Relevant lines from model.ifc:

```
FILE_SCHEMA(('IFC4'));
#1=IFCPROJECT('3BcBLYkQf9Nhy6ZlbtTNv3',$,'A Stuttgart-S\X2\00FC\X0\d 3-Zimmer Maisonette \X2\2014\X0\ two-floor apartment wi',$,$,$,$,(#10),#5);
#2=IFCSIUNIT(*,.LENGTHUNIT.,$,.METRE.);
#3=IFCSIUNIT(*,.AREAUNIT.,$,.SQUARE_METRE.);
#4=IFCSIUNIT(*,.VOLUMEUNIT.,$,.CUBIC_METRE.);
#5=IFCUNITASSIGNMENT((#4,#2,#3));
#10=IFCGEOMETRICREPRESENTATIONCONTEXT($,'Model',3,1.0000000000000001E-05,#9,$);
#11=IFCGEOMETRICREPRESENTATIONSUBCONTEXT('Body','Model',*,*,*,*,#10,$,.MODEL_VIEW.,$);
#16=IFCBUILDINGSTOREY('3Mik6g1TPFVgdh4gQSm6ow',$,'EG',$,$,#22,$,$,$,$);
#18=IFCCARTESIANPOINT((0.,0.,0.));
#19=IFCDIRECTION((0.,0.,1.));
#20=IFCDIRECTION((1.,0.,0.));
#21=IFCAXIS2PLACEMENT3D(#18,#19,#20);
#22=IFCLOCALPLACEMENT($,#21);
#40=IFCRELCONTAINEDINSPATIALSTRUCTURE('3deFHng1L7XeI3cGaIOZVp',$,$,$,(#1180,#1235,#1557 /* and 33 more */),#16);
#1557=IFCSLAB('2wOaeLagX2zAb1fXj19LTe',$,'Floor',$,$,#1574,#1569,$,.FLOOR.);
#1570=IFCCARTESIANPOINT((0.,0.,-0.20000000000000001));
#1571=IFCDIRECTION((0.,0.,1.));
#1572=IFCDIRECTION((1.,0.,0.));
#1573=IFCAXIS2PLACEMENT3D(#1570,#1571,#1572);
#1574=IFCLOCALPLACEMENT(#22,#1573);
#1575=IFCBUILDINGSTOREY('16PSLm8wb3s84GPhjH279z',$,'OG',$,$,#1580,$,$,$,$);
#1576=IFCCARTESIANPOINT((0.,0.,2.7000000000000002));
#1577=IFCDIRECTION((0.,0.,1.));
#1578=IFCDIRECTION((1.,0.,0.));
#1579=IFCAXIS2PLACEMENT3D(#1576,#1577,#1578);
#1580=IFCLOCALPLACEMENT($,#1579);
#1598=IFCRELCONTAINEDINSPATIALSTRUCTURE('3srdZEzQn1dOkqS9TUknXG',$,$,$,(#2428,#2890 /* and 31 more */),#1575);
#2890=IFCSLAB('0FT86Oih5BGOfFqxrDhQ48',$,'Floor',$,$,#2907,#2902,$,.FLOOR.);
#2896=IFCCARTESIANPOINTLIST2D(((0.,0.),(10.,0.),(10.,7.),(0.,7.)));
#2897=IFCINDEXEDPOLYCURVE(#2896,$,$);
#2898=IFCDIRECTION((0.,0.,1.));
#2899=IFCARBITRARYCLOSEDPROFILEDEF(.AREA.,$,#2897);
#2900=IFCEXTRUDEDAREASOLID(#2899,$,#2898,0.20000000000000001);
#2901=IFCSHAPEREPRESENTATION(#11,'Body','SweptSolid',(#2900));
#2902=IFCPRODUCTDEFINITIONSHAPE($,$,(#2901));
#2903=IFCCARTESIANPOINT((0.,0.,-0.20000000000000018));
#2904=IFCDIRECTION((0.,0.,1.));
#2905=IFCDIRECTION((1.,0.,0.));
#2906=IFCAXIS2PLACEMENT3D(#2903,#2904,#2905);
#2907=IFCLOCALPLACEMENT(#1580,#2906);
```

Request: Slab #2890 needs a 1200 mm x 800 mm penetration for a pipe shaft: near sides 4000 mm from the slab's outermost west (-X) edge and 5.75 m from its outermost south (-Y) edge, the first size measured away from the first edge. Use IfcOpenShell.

```python
import numpy as np
import ifcopenshell
import ifcopenshell.api.feature
import ifcopenshell.api.geometry
import ifcopenshell.api.root
import ifcopenshell.geom
import ifcopenshell.util.placement
import ifcopenshell.util.representation
import ifcopenshell.util.shape
import ifcopenshell.util.unit

model = ifcopenshell.open("model.ifc")
unit_scale = ifcopenshell.util.unit.calculate_unit_scale(model)
settings = ifcopenshell.geom.settings()


def volume(element):
    """Net volume in cubic metres, openings subtracted."""
    shape = ifcopenshell.geom.create_shape(settings, element)
    return ifcopenshell.util.shape.get_volume(shape.geometry)


slab = model.by_guid("0FT86Oih5BGOfFqxrDhQ48")
before = volume(slab)

# Extent in the slab's own axes, in metres. The edges named are its -X and -Y sides.
slab_shape = ifcopenshell.geom.create_shape(settings, slab)
vertices = ifcopenshell.util.shape.get_vertices(slab_shape.geometry)
x_min, y_min, bottom = vertices.min(axis=0)
top = vertices[:, 2].max()

opening = ifcopenshell.api.root.create_entity(model, ifc_class="IfcOpeningElement", name="Pipe shaft opening", predefined_type="OPENING")
context = ifcopenshell.util.representation.get_context(model, "Model", "Body", "MODEL_VIEW")
width, depth = 1.2, 0.8
outline = [(0.0, 0.0), (width, 0.0), (width, depth), (0.0, depth), (0.0, 0.0)]
# Overshoot both faces by 50 mm so the cut is clean.
shape = ifcopenshell.api.geometry.add_slab_representation(
    model, context=context, depth=top - bottom + 0.1, polyline=outline
)
ifcopenshell.api.geometry.assign_representation(model, product=opening, representation=shape)

matrix = ifcopenshell.util.placement.get_local_placement(slab.ObjectPlacement)
matrix[:, 3] = matrix @ np.append(np.array([x_min + 4, y_min + 5.75, bottom - 0.05]) / unit_scale, 1.0)
ifcopenshell.api.geometry.edit_object_placement(model, product=opening, matrix=matrix, is_si=False)
ifcopenshell.api.feature.add_feature(model, feature=opening, element=slab)

after = volume(slab)

print(f"slab volume {before:.3f} -> {after:.3f} m3")

model.write("model_v2.ifc")
```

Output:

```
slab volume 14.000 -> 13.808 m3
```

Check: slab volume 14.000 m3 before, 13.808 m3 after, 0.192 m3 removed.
